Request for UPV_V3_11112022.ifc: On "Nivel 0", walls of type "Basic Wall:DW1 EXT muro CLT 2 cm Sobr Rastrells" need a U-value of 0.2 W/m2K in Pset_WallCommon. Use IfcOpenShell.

First a look at what the model holds.

```python
import ifcopenshell
import ifcopenshell.util.element

model = ifcopenshell.open("UPV_V3_11112022.ifc")
print(model.schema)
storey = next(s for s in model.by_type("IfcBuildingStorey") if s.Name == "Nivel 0")
walls = [e for e in ifcopenshell.util.element.get_decomposition(storey) if e.is_a("IfcWall")]
seen = {}
for e in walls:
    element_type = ifcopenshell.util.element.get_type(e)
    key = (element_type.Name if element_type != e and element_type else None, ifcopenshell.util.element.get_pset(e, "Pset_WallCommon", "ThermalTransmittance"))
    seen[key] = seen.get(key, 0) + 1
for (name, value), count in sorted(seen.items(), key=str):
    print(count, "x", name, "|", value)
```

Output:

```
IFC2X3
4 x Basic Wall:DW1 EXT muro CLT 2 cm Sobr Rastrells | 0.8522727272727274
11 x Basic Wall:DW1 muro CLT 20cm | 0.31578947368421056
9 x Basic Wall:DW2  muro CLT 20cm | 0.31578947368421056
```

```python
import ifcopenshell
import ifcopenshell.api.pset
import ifcopenshell.util.element

model = ifcopenshell.open("UPV_V3_11112022.ifc")

storey = next(s for s in model.by_type("IfcBuildingStorey") if s.Name == "Nivel 0")
walls = [e for e in ifcopenshell.util.element.get_decomposition(storey) if e.is_a("IfcWall")]

count = 0
for e in walls:
    element_type = ifcopenshell.util.element.get_type(e)
    if element_type in (None, e) or element_type.Name != "Basic Wall:DW1 EXT muro CLT 2 cm Sobr Rastrells":
        continue
    # add_pset returns the element's existing set when there is one.
    pset = ifcopenshell.api.pset.add_pset(model, product=e, name="Pset_WallCommon")
    ifcopenshell.api.pset.edit_pset(model, pset=pset, properties={"ThermalTransmittance": 0.2})
    count += 1

print(count, "walls updated")

model.write("UPV_V3_11112022_rev.ifc")
```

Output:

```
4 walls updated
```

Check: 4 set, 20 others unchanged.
